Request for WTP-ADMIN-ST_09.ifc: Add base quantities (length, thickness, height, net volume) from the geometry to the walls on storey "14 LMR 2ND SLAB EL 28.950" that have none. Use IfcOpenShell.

First a look at what the model holds.

```python
import ifcopenshell
import ifcopenshell.util.element
import ifcopenshell.util.unit

model = ifcopenshell.open("WTP-ADMIN-ST_09.ifc")
print(model.schema)
for unit_type in ("LENGTHUNIT", "AREAUNIT", "VOLUMEUNIT"):
    print(unit_type, ifcopenshell.util.unit.calculate_unit_scale(model, unit_type))
storey = next(s for s in model.by_type("IfcBuildingStorey") if s.Name == "14 LMR 2ND SLAB EL 28.950")
walls = [e for e in ifcopenshell.util.element.get_decomposition(storey) if e.is_a("IfcWall")]
for e in sorted(walls, key=lambda e: e.id()):
    print(e.id(), e.is_a(), e.Name, list(ifcopenshell.util.element.get_psets(e, qtos_only=True)), sep=" | ")
```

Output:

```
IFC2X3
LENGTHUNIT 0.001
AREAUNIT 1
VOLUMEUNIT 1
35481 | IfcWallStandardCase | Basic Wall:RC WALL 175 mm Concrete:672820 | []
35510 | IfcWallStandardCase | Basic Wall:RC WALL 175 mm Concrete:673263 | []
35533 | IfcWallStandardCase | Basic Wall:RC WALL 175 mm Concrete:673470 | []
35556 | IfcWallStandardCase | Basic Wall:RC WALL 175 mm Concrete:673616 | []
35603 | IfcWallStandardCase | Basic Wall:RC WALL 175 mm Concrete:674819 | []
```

```python
import ifcopenshell
import ifcopenshell.api.pset
import ifcopenshell.geom
import ifcopenshell.util.element
import ifcopenshell.util.shape
import ifcopenshell.util.unit

model = ifcopenshell.open("WTP-ADMIN-ST_09.ifc")
unit_scale = ifcopenshell.util.unit.calculate_unit_scale(model)
volume_scale = ifcopenshell.util.unit.calculate_unit_scale(model, "VOLUMEUNIT")
settings = ifcopenshell.geom.settings()

storey = next(s for s in model.by_type("IfcBuildingStorey") if s.Name == "14 LMR 2ND SLAB EL 28.950")
walls = [e for e in ifcopenshell.util.element.get_decomposition(storey) if e.is_a("IfcWall")]

for e in sorted(walls, key=lambda e: e.id()):
    if ifcopenshell.util.element.get_psets(e, qtos_only=True, should_inherit=False):
        continue
    # Geometry comes back in metres, in the element's own axes.
    shape = ifcopenshell.geom.create_shape(settings, e)
    values = {
        "Length": ifcopenshell.util.shape.get_x(shape.geometry) / unit_scale,
        "Width": ifcopenshell.util.shape.get_y(shape.geometry) / unit_scale,
        "Height": ifcopenshell.util.shape.get_z(shape.geometry) / unit_scale,
        "NetVolume": ifcopenshell.util.shape.get_volume(shape.geometry) / volume_scale,
    }
    qto = ifcopenshell.api.pset.add_qto(model, product=e, name="BaseQuantities")
    ifcopenshell.api.pset.edit_qto(model, qto=qto, properties=values)
    print(e.id(), {k: round(v, 3) for k, v in values.items()})

model.write("WTP-ADMIN-ST_09-out.ifc")
```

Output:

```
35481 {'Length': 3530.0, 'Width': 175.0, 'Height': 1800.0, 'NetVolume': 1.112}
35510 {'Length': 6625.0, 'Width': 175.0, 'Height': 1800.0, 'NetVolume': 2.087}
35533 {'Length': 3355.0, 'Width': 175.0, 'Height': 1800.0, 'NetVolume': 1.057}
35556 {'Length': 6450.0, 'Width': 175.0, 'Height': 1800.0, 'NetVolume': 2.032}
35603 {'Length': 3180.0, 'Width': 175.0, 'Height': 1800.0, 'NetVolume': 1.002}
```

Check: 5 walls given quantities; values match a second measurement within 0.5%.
